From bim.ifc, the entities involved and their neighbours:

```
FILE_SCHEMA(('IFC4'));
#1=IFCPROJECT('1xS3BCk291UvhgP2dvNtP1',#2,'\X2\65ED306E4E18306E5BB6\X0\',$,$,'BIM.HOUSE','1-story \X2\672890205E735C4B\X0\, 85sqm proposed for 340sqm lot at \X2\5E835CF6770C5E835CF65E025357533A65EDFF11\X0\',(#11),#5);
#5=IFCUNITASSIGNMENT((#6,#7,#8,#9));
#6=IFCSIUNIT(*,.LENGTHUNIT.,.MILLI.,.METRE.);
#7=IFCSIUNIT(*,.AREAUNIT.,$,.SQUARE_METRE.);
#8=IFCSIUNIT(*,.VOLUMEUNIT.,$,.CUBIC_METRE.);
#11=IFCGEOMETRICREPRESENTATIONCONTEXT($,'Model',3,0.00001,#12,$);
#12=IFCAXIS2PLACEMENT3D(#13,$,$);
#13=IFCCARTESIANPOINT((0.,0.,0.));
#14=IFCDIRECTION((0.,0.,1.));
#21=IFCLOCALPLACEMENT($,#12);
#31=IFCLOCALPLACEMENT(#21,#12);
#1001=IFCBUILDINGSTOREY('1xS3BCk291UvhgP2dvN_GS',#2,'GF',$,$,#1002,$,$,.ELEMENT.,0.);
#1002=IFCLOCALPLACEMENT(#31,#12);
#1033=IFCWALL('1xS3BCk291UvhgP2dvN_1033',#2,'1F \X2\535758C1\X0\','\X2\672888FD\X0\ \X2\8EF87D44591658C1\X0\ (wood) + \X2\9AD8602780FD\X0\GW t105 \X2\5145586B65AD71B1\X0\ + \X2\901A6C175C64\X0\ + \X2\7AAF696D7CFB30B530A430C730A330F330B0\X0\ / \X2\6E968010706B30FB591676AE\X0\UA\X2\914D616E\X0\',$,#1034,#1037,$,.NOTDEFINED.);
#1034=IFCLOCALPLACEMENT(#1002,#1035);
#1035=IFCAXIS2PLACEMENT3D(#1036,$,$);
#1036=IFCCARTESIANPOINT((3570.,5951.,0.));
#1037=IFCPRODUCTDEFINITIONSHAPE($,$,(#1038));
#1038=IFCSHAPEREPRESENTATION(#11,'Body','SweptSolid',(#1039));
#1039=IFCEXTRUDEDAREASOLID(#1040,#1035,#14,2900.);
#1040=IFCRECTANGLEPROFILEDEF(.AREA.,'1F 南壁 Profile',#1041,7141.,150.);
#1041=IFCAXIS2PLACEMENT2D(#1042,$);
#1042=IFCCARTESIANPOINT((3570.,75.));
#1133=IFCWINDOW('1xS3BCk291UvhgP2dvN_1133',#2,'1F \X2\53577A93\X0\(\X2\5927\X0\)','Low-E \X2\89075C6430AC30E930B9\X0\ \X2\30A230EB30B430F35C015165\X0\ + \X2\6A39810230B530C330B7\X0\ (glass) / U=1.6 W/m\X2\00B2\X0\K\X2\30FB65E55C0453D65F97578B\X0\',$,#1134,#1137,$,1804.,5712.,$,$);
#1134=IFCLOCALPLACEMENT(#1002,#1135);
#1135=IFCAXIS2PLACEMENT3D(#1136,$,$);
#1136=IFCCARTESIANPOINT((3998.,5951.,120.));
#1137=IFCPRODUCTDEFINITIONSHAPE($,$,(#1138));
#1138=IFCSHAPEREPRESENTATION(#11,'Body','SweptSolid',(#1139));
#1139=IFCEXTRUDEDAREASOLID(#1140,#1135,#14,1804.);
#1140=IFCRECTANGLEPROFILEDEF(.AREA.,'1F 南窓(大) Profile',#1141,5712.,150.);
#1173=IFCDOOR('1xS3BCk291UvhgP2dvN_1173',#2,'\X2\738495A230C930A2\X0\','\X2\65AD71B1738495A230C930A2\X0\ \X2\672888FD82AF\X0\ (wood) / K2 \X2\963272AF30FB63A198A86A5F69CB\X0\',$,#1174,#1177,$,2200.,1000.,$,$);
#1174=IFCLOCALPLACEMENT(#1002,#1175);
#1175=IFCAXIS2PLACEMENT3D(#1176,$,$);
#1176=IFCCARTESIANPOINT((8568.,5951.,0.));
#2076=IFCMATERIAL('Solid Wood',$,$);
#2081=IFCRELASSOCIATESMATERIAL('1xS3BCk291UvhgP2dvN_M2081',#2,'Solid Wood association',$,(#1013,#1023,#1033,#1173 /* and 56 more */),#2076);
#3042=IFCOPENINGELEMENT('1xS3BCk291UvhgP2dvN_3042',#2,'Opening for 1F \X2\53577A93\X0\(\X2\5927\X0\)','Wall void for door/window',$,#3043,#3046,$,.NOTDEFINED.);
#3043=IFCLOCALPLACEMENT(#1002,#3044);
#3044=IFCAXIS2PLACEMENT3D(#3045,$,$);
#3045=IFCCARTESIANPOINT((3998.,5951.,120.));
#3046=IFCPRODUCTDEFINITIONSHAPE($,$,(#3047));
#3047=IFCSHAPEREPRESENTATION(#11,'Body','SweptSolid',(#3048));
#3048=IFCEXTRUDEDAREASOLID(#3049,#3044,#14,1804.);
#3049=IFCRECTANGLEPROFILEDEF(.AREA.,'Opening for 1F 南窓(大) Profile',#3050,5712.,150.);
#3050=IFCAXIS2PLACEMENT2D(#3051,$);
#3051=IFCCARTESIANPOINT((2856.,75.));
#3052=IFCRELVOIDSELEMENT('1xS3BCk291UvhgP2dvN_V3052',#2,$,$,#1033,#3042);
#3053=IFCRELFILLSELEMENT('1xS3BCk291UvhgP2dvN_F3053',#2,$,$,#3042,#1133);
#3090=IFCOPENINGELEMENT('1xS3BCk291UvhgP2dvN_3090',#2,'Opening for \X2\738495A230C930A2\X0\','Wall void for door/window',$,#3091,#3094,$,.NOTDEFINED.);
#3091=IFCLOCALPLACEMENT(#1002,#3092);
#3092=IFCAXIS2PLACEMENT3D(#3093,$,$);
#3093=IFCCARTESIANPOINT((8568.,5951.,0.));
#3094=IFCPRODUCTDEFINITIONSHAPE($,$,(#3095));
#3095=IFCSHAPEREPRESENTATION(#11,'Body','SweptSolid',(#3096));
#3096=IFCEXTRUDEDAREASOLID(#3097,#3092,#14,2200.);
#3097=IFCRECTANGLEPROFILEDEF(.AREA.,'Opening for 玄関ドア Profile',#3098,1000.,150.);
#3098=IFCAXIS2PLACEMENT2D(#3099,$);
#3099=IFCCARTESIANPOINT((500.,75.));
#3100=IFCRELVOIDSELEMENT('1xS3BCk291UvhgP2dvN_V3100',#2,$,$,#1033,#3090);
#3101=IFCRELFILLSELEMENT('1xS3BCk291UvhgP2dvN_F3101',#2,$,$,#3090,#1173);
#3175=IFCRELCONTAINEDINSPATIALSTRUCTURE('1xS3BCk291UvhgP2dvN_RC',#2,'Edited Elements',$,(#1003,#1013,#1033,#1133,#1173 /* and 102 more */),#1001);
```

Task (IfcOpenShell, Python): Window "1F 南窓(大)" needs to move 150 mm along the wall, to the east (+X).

```python
import ifcopenshell
import ifcopenshell.api.geometry
import ifcopenshell.util.placement
import ifcopenshell.util.unit

model = ifcopenshell.open("bim.ifc")
unit_scale = ifcopenshell.util.unit.calculate_unit_scale(model)

window = model.by_guid("1xS3BCk291UvhgP2dvN_1133")
opening = window.FillsVoids[0].RelatingOpeningElement
wall = opening.VoidsElements[0].RelatingBuildingElement

wall_matrix = ifcopenshell.util.placement.get_local_placement(wall.ObjectPlacement)
shift = wall_matrix[:3, 0] * 0.15 / unit_scale
before = ifcopenshell.util.placement.get_local_placement(window.ObjectPlacement)[:3, 3].copy()

# The window is not placed relative to its opening, so move both.
for product in (opening, window):
    matrix = ifcopenshell.util.placement.get_local_placement(product.ObjectPlacement)
    matrix[:3, 3] += shift
    ifcopenshell.api.geometry.edit_object_placement(model, product=product, matrix=matrix, is_si=False)

after = ifcopenshell.util.placement.get_local_placement(window.ObjectPlacement)[:3, 3]
print("window moved by", (after - before).round(3) + 0.0)

model.write("bim_rev.ifc")
```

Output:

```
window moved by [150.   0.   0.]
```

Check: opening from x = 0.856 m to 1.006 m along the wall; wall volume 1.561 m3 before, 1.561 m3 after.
